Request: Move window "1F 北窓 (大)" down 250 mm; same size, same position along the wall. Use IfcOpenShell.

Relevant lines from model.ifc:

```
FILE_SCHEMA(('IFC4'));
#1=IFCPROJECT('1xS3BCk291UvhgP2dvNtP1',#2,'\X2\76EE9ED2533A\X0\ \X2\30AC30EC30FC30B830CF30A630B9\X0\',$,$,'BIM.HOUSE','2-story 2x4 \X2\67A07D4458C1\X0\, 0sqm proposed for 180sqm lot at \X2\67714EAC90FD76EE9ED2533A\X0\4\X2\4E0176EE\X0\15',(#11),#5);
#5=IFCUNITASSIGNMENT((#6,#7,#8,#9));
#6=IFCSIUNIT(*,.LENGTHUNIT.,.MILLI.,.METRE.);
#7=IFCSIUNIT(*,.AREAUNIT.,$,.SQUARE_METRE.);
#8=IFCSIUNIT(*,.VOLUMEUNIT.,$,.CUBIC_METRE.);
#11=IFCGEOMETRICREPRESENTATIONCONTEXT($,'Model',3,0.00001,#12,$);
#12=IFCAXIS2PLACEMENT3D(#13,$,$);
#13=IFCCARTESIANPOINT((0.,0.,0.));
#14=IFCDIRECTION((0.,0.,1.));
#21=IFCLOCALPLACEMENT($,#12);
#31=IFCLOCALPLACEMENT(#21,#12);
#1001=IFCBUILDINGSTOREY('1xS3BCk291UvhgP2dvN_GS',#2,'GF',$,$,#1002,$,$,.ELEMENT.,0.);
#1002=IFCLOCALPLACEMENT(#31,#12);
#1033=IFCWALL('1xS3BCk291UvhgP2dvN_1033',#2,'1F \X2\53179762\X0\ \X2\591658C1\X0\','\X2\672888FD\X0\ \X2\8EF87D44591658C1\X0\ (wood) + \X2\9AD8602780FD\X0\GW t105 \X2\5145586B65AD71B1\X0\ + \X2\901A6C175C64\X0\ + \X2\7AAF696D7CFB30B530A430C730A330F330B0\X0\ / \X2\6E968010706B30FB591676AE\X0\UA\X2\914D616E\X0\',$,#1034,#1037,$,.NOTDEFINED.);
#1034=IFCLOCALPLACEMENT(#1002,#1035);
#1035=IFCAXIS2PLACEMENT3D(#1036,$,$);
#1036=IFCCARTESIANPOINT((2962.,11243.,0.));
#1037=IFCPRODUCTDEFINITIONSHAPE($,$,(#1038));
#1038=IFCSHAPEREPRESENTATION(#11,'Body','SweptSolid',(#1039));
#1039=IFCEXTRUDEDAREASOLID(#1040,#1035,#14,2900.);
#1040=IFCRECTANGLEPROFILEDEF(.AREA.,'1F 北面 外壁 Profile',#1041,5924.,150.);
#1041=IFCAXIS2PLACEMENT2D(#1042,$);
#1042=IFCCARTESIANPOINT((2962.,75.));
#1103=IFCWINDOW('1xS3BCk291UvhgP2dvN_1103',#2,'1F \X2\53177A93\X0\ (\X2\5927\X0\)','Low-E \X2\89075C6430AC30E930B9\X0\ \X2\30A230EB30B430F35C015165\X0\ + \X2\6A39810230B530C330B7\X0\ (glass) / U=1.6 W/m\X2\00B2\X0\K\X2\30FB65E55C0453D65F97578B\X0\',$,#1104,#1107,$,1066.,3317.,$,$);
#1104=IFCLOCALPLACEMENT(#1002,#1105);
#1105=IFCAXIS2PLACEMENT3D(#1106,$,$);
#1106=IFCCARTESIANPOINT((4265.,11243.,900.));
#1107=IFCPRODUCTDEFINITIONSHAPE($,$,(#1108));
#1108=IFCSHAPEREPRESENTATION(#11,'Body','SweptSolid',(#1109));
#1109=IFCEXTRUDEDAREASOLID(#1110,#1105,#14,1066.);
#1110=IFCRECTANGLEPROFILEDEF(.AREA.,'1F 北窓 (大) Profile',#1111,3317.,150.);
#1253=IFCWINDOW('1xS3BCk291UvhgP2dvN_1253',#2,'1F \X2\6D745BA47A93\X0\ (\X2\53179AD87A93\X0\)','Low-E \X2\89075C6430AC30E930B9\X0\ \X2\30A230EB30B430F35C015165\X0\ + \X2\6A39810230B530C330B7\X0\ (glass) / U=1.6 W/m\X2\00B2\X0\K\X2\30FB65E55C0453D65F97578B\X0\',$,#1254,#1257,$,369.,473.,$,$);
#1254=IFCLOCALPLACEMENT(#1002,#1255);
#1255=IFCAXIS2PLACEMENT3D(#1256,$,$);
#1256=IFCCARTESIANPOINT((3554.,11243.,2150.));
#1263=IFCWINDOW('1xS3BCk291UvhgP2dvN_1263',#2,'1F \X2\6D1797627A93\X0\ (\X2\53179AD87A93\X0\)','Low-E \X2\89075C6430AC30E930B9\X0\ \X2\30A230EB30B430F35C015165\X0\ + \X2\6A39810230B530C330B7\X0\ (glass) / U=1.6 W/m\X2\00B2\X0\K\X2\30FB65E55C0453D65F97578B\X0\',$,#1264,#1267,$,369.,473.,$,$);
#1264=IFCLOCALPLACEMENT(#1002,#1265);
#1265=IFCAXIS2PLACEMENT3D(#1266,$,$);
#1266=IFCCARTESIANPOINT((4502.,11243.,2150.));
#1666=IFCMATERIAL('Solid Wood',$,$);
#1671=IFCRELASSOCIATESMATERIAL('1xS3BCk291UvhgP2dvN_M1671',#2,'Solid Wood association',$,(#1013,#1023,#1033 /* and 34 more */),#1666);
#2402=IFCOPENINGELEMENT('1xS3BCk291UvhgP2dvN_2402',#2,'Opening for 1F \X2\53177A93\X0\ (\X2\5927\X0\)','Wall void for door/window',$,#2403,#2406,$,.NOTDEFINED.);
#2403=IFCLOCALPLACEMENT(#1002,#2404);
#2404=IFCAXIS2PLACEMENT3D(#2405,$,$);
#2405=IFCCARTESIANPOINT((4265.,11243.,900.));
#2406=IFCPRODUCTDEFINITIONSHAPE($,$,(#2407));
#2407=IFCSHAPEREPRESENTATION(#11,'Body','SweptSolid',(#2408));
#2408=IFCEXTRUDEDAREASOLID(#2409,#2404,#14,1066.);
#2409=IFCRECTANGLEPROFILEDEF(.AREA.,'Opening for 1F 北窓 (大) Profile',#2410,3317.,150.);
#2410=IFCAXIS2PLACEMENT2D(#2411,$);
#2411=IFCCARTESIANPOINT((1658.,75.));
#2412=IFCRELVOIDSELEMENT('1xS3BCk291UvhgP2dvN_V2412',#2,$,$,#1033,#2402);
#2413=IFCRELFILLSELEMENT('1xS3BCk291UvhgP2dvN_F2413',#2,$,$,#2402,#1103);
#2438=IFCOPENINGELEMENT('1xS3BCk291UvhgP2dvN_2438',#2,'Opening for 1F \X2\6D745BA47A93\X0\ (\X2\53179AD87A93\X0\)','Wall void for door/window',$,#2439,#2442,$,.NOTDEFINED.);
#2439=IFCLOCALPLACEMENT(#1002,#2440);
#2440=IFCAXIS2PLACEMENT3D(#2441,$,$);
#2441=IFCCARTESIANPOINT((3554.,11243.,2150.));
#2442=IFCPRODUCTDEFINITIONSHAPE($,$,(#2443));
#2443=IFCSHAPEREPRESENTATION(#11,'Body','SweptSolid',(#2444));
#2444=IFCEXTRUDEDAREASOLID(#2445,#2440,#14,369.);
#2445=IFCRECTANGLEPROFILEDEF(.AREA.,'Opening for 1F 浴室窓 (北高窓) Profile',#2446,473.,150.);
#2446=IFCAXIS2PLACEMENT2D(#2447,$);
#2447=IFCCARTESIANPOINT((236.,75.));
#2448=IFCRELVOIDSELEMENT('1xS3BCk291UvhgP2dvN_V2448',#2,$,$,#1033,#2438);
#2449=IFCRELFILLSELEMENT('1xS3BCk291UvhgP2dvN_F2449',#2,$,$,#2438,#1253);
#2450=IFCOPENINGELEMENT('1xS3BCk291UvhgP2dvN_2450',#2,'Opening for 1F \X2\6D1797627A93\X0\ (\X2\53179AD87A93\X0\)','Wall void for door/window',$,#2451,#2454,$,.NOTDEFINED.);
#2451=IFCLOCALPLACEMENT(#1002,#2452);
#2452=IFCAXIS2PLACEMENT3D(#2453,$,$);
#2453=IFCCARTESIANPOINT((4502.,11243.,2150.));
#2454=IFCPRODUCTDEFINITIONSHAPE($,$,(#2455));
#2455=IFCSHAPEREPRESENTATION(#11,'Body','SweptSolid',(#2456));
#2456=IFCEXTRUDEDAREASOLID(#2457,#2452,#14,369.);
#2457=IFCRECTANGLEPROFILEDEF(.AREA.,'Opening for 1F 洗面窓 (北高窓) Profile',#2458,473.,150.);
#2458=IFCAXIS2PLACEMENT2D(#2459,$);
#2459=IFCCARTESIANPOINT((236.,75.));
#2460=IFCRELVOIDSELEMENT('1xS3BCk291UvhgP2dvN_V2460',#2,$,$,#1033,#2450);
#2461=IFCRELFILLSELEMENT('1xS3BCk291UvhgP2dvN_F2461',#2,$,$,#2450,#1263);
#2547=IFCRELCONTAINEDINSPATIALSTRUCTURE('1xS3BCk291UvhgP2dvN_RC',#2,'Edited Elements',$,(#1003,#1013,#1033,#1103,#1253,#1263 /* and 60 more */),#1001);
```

```python
import numpy as np
import ifcopenshell
import ifcopenshell.api.geometry
import ifcopenshell.util.placement
import ifcopenshell.util.unit

model = ifcopenshell.open("model.ifc")
unit_scale = ifcopenshell.util.unit.calculate_unit_scale(model)

window = model.by_guid("1xS3BCk291UvhgP2dvN_1103")
opening = window.FillsVoids[0].RelatingOpeningElement
dz = -250.0

shift = np.array([0.0, 0.0, dz])
# The window is not placed relative to its opening, so move both.
for product in (opening, window):
    matrix = ifcopenshell.util.placement.get_local_placement(product.ObjectPlacement)
    matrix[:3, 3] += shift
    ifcopenshell.api.geometry.edit_object_placement(model, product=product, matrix=matrix, is_si=False)

print(f"moved by {dz * unit_scale:+.3f} m")

model.write("model_rev.ifc")
```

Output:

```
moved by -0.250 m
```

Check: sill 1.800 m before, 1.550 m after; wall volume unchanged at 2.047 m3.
